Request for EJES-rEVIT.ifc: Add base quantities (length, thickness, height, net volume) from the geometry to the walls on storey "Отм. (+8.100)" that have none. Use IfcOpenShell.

First a look at what the model holds.

```python
import ifcopenshell
import ifcopenshell.util.element
import ifcopenshell.util.unit

model = ifcopenshell.open("EJES-rEVIT.ifc")
print(model.schema)
for unit_type in ("LENGTHUNIT", "AREAUNIT", "VOLUMEUNIT"):
    print(unit_type, ifcopenshell.util.unit.calculate_unit_scale(model, unit_type))
storey = next(s for s in model.by_type("IfcBuildingStorey") if s.Name == "Отм. (+8.100)")
walls = [e for e in ifcopenshell.util.element.get_decomposition(storey) if e.is_a("IfcWall")]
for e in sorted(walls, key=lambda e: e.id()):
    print(e.id(), e.is_a(), e.Name, list(ifcopenshell.util.element.get_psets(e, qtos_only=True)), sep=" | ")
```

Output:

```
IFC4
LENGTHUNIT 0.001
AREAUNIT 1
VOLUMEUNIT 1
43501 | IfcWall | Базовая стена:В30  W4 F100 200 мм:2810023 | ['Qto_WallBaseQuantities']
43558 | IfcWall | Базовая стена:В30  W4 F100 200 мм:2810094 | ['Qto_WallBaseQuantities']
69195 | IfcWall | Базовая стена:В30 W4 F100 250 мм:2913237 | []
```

```python
import ifcopenshell
import ifcopenshell.api.pset
import ifcopenshell.geom
import ifcopenshell.util.element
import ifcopenshell.util.shape
import ifcopenshell.util.unit

model = ifcopenshell.open("EJES-rEVIT.ifc")
unit_scale = ifcopenshell.util.unit.calculate_unit_scale(model)
volume_scale = ifcopenshell.util.unit.calculate_unit_scale(model, "VOLUMEUNIT")
settings = ifcopenshell.geom.settings()

storey = next(s for s in model.by_type("IfcBuildingStorey") if s.Name == "Отм. (+8.100)")
walls = [e for e in ifcopenshell.util.element.get_decomposition(storey) if e.is_a("IfcWall")]

for e in sorted(walls, key=lambda e: e.id()):
    if ifcopenshell.util.element.get_psets(e, qtos_only=True, should_inherit=False):
        continue
    # Geometry comes back in metres, in the element's own axes.
    shape = ifcopenshell.geom.create_shape(settings, e)
    values = {
        "Length": ifcopenshell.util.shape.get_x(shape.geometry) / unit_scale,
        "Width": ifcopenshell.util.shape.get_y(shape.geometry) / unit_scale,
        "Height": ifcopenshell.util.shape.get_z(shape.geometry) / unit_scale,
        "NetVolume": ifcopenshell.util.shape.get_volume(shape.geometry) / volume_scale,
    }
    qto = ifcopenshell.api.pset.add_qto(model, product=e, name="Qto_WallBaseQuantities")
    ifcopenshell.api.pset.edit_qto(model, qto=qto, properties=values)
    print(e.id(), {k: round(v, 3) for k, v in values.items()})

model.write("EJES-rEVIT_edited.ifc")
```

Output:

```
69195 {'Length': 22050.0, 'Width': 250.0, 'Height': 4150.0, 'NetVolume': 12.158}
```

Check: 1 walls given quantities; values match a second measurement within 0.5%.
